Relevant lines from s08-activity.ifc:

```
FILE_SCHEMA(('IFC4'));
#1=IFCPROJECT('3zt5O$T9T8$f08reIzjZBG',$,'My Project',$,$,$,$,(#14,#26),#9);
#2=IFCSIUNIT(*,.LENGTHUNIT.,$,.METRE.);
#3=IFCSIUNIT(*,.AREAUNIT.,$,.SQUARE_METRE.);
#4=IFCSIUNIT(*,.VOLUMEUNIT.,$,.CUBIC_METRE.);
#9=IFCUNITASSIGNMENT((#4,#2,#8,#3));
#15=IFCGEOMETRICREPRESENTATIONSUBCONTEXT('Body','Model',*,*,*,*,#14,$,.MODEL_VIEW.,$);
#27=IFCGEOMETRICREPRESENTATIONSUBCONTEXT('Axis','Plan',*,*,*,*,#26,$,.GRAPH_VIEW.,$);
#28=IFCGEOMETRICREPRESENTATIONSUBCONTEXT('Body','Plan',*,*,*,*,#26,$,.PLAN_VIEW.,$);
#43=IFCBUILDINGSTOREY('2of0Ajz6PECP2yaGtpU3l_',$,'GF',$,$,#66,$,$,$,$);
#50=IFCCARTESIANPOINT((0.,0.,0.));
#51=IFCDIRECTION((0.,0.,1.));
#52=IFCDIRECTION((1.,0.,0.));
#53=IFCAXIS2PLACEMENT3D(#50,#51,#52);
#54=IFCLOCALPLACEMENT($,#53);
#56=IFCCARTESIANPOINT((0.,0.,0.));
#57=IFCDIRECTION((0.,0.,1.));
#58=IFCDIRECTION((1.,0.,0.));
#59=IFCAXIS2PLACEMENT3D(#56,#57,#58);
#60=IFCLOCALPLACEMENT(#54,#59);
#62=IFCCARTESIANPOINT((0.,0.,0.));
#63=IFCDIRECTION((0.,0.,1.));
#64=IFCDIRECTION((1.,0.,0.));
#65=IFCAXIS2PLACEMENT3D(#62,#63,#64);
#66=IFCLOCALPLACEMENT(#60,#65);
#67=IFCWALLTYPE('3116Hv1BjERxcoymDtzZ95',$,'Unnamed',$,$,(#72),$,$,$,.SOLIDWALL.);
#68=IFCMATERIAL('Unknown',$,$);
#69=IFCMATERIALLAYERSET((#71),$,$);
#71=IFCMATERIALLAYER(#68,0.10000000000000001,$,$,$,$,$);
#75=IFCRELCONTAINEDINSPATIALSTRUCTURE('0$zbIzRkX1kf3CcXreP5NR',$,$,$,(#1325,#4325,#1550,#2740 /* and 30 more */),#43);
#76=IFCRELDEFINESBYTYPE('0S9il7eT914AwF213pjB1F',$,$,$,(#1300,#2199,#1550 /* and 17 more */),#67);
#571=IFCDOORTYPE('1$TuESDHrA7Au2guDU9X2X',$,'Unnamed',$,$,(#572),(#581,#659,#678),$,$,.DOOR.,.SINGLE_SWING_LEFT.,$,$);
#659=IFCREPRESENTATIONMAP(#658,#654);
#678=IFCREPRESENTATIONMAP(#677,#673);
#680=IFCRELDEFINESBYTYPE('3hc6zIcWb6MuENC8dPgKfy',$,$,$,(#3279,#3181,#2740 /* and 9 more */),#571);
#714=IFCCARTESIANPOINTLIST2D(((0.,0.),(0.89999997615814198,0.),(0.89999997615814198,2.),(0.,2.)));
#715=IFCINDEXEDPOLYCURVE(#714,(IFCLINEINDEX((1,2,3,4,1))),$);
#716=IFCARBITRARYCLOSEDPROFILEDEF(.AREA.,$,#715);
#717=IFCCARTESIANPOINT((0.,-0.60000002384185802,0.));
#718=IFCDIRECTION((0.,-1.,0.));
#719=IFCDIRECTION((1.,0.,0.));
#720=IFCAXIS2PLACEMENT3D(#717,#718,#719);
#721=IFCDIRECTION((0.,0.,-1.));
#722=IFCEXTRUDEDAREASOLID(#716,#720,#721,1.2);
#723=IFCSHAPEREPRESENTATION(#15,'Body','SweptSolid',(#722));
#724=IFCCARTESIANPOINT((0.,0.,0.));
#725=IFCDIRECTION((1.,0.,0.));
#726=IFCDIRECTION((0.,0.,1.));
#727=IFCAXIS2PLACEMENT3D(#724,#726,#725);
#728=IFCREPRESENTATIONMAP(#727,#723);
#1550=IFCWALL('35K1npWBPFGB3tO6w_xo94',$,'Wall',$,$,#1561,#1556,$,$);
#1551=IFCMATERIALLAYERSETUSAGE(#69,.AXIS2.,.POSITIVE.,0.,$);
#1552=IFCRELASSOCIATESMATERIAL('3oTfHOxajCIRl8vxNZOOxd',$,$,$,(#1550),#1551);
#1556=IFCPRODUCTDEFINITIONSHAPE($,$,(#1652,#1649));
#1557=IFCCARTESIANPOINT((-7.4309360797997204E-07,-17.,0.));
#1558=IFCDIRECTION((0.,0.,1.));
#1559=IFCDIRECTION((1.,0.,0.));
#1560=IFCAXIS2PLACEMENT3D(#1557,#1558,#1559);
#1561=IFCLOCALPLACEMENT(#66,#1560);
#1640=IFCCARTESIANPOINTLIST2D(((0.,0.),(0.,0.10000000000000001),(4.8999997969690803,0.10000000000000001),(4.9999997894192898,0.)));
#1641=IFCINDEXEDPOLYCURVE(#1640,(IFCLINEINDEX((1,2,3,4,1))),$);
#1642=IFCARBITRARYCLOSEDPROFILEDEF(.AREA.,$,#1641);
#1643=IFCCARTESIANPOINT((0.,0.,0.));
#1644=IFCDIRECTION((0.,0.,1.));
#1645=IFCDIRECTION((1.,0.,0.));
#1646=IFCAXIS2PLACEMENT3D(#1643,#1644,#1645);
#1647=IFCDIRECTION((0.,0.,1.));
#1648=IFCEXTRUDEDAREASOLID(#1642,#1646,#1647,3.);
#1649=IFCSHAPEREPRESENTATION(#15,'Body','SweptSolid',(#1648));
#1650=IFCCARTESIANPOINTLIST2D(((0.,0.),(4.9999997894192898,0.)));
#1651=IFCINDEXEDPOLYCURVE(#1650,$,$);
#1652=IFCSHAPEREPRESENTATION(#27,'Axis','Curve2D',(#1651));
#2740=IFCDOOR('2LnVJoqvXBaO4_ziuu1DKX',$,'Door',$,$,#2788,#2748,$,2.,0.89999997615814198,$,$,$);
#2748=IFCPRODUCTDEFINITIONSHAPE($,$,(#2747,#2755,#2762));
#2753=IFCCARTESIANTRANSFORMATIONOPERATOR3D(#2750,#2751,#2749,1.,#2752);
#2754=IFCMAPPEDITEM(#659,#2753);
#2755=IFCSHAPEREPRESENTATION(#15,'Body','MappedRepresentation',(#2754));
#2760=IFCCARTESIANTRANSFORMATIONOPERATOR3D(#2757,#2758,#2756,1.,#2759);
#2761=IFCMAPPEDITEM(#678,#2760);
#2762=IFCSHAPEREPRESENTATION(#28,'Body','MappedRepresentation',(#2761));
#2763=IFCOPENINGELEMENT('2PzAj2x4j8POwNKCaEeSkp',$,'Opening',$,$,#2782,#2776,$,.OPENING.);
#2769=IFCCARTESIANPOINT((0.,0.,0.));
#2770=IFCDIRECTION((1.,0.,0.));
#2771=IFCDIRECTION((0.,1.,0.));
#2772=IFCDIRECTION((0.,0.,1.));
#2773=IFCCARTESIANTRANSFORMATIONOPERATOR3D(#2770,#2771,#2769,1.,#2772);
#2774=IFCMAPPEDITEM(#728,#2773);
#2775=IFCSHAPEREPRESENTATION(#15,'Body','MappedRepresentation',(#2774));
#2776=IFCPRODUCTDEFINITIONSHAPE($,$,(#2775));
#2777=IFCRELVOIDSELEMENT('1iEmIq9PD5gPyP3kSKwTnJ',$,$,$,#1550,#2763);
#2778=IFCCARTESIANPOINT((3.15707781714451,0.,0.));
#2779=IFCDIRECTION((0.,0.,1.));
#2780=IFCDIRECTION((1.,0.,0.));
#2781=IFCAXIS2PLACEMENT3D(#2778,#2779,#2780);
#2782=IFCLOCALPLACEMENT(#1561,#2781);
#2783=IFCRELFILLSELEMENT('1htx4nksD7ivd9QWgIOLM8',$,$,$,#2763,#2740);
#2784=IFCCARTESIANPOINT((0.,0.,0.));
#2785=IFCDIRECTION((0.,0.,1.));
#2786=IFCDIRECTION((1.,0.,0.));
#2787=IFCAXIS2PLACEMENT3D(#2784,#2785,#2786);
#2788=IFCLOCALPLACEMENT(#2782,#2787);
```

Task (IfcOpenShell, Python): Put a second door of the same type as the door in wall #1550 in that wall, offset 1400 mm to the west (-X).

```python
import ifcopenshell
import ifcopenshell.api.feature
import ifcopenshell.api.geometry
import ifcopenshell.api.root
import ifcopenshell.geom
import ifcopenshell.util.element
import ifcopenshell.util.placement
import ifcopenshell.util.shape
import ifcopenshell.util.unit

model = ifcopenshell.open("s08-activity.ifc")
unit_scale = ifcopenshell.util.unit.calculate_unit_scale(model)
settings = ifcopenshell.geom.settings()


def volume(element):
    """Net volume in cubic metres, openings subtracted."""
    shape = ifcopenshell.geom.create_shape(settings, element)
    return ifcopenshell.util.shape.get_volume(shape.geometry)


door = model.by_id(2740)
opening = door.FillsVoids[0].RelatingOpeningElement
wall = opening.VoidsElements[0].RelatingBuildingElement
before = volume(wall)
shift = ifcopenshell.util.placement.get_local_placement(wall.ObjectPlacement)[:3, 0] * -1.4 / unit_scale

# copy_class copies the void relationship, type, container and properties, but no geometry.
new_opening = ifcopenshell.api.root.copy_class(model, product=opening)
new_opening.Representation = ifcopenshell.util.element.copy_deep(
    model, opening.Representation, exclude=["IfcGeometricRepresentationContext", "IfcRepresentationMap"]
)
new_door = ifcopenshell.api.root.copy_class(model, product=door)
new_door.Representation = ifcopenshell.util.element.copy_deep(
    model, door.Representation, exclude=["IfcGeometricRepresentationContext", "IfcRepresentationMap"]
)
ifcopenshell.api.feature.add_filling(model, opening=new_opening, element=new_door)

for old, new in ((opening, new_opening), (door, new_door)):
    matrix = ifcopenshell.util.placement.get_local_placement(old.ObjectPlacement)
    matrix[:3, 3] += shift
    ifcopenshell.api.geometry.edit_object_placement(model, product=new, matrix=matrix, is_si=False)

after = volume(wall)

print(f"wall volume {before:.3f} -> {after:.3f} m3")

model.write("s08-activity_v2.ifc")
```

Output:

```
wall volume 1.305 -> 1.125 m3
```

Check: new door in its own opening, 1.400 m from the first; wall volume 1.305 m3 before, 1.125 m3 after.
